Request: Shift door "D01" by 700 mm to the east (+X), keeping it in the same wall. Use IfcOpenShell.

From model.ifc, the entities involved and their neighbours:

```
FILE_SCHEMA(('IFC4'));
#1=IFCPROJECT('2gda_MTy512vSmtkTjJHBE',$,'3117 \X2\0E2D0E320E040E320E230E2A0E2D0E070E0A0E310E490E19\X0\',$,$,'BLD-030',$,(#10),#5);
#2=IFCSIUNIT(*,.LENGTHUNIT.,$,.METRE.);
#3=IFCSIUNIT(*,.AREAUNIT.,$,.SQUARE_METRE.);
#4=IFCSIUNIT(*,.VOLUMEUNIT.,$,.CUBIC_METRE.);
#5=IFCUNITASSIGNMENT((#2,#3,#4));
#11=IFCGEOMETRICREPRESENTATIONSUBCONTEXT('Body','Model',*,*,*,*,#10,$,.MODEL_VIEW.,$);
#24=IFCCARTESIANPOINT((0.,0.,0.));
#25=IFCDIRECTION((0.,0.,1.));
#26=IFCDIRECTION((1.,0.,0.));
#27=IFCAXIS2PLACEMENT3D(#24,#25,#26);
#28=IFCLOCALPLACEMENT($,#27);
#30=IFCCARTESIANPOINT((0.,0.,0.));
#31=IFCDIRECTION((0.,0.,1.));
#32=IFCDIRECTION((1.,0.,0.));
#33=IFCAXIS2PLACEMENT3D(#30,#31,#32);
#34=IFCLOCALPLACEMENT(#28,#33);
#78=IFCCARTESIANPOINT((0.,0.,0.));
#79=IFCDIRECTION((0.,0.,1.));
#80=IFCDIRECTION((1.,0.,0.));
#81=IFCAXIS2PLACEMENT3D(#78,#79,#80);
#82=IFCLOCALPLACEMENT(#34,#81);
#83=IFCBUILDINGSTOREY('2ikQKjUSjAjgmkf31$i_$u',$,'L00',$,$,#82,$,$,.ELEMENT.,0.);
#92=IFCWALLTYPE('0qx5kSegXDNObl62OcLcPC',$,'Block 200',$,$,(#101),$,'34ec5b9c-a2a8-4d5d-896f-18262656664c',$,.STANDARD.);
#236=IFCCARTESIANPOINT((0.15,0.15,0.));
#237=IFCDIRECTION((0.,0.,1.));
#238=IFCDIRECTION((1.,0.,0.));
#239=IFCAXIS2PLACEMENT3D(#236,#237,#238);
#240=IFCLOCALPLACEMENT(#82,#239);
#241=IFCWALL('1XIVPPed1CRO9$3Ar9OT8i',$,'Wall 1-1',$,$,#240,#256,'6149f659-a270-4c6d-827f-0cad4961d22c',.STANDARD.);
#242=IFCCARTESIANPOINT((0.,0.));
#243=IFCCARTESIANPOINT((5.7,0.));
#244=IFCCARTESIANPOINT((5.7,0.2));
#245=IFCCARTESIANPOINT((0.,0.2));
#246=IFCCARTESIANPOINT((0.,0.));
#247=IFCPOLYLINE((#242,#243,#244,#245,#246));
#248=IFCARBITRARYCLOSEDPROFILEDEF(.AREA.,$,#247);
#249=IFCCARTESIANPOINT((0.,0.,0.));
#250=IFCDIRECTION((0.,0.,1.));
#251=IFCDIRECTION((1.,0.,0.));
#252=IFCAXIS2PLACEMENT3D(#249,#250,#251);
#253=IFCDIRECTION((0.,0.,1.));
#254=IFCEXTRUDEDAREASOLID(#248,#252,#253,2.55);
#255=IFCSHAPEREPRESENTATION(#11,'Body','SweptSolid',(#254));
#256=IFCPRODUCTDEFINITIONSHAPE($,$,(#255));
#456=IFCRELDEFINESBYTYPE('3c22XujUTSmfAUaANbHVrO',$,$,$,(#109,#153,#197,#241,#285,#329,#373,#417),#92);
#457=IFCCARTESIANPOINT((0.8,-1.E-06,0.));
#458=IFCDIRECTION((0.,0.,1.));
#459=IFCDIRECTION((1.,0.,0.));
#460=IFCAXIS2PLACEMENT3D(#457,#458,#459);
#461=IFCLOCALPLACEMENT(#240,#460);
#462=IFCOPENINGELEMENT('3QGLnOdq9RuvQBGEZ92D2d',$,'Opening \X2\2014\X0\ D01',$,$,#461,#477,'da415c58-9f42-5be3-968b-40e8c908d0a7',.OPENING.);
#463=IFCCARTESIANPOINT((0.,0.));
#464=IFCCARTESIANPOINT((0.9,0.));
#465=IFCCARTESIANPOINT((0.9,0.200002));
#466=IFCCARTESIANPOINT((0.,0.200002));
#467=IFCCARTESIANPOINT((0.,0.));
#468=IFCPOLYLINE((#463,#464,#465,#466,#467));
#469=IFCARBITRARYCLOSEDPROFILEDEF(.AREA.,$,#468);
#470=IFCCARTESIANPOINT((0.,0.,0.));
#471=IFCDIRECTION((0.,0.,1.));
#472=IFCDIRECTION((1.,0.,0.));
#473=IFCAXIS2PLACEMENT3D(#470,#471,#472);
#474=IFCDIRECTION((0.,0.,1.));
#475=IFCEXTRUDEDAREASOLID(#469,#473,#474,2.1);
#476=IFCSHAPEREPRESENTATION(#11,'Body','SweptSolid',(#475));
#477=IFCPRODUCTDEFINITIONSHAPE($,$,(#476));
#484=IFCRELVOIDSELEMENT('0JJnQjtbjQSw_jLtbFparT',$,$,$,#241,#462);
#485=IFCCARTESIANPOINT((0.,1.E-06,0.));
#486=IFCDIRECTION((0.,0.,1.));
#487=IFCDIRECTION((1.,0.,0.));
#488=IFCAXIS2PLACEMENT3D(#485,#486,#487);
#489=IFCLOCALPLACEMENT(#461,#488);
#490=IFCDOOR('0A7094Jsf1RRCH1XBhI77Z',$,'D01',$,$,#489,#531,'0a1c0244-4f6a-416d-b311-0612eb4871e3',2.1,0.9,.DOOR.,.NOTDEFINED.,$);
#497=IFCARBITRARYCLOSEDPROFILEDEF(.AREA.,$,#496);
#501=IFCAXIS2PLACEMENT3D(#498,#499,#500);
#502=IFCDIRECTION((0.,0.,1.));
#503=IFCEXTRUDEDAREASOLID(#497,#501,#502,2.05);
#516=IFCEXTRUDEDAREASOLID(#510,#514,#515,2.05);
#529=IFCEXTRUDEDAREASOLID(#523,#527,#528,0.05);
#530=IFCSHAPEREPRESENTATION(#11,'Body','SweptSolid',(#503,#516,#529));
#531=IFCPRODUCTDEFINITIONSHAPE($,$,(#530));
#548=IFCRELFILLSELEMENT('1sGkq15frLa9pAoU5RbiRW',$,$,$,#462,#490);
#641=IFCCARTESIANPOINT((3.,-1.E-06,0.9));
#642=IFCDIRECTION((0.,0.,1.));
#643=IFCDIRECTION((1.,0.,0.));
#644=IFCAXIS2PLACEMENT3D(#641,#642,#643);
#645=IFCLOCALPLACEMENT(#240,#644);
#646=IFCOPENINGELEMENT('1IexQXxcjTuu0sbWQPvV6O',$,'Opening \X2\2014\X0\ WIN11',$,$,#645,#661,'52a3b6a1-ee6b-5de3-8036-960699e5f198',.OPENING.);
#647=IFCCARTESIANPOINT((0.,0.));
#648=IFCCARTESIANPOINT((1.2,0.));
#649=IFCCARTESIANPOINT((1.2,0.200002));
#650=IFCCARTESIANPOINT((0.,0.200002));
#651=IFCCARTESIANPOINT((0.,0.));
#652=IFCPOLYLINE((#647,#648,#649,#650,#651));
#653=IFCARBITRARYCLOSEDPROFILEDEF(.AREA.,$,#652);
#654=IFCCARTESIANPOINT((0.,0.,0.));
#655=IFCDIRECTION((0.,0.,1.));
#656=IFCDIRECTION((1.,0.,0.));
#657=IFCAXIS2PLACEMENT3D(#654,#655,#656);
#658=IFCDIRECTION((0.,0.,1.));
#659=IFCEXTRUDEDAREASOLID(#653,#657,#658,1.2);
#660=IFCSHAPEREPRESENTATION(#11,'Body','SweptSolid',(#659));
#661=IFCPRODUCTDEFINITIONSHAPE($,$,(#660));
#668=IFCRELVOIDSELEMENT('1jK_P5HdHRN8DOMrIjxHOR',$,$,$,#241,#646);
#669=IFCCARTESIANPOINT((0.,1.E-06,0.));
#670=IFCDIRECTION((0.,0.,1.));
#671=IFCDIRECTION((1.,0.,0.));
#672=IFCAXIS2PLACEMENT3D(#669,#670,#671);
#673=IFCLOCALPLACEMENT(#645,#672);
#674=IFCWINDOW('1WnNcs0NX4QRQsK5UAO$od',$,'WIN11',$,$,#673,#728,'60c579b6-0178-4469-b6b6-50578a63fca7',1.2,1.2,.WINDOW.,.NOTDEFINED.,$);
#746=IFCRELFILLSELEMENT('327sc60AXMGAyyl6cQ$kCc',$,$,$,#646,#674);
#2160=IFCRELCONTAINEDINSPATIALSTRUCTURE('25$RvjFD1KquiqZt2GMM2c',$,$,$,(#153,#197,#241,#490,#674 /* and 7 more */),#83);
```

```python
import ifcopenshell
import ifcopenshell.api.geometry
import ifcopenshell.util.placement

model = ifcopenshell.open("model.ifc")

door = model.by_id(490)
opening = door.FillsVoids[0].RelatingOpeningElement
wall = opening.VoidsElements[0].RelatingBuildingElement

wall_matrix = ifcopenshell.util.placement.get_local_placement(wall.ObjectPlacement)
shift = wall_matrix[:3, 0] * 0.7
before = ifcopenshell.util.placement.get_local_placement(door.ObjectPlacement)[:3, 3].copy()

# The door is placed relative to its opening, so it follows when the opening moves.
matrix = ifcopenshell.util.placement.get_local_placement(opening.ObjectPlacement)
matrix[:3, 3] += shift
ifcopenshell.api.geometry.edit_object_placement(
    model, product=opening, matrix=matrix, is_si=False, should_transform_children=True
)

after = ifcopenshell.util.placement.get_local_placement(door.ObjectPlacement)[:3, 3]
print("door moved by", (after - before).round(3) + 0.0)

model.write("model_rev.ifc")
```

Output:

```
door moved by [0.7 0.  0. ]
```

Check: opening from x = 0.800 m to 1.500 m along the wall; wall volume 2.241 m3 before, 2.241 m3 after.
